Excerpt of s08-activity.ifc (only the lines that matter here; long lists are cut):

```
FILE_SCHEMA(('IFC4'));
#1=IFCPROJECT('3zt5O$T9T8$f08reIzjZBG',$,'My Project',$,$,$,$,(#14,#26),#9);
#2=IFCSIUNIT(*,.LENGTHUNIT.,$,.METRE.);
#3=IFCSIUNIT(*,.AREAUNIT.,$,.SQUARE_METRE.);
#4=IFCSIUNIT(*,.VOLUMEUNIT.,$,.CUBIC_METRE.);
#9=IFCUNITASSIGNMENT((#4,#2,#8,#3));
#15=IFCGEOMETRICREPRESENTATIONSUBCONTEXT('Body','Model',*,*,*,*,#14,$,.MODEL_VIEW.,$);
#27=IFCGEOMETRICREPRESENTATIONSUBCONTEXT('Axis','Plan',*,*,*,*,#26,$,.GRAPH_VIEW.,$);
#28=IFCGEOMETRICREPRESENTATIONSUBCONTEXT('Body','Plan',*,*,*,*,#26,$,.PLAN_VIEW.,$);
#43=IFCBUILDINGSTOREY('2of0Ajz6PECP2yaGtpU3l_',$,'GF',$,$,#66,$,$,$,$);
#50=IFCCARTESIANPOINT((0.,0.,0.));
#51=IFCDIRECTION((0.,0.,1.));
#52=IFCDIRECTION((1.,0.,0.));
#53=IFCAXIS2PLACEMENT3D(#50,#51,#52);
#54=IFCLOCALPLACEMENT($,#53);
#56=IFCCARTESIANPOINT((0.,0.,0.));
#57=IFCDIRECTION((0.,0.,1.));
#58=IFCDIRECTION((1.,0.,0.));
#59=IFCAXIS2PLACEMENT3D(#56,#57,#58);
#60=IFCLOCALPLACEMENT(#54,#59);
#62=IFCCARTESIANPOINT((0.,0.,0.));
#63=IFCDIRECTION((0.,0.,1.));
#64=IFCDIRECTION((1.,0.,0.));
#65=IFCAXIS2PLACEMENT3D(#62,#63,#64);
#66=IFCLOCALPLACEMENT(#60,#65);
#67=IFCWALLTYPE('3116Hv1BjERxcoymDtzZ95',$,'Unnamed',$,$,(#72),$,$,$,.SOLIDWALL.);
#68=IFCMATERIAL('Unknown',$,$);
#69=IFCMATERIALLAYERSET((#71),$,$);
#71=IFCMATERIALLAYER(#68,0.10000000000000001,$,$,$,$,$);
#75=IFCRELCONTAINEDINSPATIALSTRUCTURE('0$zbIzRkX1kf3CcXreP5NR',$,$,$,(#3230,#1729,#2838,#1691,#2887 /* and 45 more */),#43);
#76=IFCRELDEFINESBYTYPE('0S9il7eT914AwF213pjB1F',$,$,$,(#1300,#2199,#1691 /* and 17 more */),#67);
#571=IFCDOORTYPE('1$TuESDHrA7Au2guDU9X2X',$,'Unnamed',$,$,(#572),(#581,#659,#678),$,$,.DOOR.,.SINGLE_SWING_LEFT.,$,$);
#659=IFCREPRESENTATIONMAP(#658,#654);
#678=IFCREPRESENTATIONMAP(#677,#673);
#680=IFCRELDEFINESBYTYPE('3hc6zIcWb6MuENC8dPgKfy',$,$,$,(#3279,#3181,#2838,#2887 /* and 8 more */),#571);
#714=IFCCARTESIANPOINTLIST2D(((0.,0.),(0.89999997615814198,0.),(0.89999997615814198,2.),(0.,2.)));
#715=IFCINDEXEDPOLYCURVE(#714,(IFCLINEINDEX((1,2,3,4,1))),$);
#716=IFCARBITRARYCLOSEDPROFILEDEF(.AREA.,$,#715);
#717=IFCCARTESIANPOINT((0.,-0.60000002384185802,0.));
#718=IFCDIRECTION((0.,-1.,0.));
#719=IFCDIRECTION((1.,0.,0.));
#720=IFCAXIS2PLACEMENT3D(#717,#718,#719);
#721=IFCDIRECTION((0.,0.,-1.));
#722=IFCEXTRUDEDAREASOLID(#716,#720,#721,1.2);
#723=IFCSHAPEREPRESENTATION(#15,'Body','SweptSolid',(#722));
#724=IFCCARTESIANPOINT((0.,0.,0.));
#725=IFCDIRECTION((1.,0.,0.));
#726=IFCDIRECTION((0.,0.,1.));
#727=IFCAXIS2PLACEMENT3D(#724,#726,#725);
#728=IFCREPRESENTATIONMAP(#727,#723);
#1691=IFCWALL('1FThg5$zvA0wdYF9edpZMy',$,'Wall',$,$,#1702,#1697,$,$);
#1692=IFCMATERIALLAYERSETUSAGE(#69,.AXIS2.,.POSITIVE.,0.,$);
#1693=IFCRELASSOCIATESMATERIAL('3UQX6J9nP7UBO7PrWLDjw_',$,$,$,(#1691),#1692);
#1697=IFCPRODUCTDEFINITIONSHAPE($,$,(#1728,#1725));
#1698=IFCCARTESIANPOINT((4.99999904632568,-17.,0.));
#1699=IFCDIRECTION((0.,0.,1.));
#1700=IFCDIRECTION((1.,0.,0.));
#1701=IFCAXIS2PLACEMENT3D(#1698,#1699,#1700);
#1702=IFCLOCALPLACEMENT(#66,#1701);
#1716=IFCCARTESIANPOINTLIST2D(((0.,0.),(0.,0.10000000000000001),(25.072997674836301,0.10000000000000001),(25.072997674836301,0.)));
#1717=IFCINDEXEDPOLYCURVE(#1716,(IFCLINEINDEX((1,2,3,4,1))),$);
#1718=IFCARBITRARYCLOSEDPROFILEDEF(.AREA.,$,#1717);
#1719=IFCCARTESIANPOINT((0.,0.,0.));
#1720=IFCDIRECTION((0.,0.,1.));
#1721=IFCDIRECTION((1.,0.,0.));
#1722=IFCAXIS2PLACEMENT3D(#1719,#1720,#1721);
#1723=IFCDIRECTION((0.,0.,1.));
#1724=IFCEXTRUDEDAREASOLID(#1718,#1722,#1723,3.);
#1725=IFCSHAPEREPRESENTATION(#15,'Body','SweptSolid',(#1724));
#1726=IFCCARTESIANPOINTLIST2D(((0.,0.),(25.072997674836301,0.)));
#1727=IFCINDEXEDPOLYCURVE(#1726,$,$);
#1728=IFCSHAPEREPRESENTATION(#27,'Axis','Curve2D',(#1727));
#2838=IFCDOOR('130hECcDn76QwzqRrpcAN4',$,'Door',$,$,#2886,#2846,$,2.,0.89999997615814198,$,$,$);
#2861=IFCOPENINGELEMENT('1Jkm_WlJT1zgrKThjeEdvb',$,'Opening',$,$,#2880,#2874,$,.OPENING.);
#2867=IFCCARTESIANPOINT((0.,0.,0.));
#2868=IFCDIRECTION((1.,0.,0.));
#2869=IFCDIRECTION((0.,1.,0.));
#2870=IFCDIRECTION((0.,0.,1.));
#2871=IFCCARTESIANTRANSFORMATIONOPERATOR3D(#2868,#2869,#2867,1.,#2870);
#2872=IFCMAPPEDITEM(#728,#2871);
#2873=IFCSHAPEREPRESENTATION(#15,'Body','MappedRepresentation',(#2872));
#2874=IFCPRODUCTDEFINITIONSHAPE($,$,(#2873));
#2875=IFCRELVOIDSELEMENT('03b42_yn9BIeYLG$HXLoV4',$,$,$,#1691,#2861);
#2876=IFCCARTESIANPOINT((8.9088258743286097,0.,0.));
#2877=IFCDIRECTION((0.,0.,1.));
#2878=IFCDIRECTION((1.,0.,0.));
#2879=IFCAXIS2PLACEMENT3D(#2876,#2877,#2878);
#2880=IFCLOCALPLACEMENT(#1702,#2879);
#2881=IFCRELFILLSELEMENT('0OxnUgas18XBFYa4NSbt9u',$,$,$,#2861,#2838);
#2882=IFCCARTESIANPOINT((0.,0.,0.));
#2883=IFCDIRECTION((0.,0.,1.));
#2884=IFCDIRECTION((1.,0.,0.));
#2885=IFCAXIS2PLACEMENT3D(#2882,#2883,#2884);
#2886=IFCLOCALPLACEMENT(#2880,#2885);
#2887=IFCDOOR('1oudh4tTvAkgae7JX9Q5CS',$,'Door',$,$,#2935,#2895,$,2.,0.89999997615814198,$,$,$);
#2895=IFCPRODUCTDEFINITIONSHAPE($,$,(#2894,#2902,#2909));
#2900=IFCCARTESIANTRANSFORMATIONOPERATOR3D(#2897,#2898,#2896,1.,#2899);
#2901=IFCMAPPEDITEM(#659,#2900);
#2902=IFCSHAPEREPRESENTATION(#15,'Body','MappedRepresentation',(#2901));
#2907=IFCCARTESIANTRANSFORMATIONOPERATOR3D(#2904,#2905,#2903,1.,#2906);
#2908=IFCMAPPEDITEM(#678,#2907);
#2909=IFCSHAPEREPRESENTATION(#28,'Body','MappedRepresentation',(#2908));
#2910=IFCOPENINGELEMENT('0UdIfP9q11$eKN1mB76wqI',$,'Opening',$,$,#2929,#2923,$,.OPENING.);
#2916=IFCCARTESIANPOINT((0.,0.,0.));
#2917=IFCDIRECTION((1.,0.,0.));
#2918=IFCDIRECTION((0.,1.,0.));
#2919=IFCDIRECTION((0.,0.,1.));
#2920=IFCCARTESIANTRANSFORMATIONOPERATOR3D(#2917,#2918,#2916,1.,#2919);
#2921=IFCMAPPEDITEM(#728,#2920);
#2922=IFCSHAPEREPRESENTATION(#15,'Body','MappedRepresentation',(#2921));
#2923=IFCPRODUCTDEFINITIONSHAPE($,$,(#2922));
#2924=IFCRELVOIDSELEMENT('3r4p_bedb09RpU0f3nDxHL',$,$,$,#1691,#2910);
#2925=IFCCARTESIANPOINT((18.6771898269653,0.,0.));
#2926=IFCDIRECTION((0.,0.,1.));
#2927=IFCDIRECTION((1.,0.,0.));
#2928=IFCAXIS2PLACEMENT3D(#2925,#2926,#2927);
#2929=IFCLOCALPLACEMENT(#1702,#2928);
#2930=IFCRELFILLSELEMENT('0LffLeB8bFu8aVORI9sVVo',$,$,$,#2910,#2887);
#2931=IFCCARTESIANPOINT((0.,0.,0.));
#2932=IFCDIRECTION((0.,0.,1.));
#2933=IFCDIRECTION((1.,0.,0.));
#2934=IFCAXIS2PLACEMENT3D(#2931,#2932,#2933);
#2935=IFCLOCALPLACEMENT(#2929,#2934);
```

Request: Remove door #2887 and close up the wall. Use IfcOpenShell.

```python
import ifcopenshell
import ifcopenshell.api.feature
import ifcopenshell.api.root
import ifcopenshell.geom
import ifcopenshell.util.shape

model = ifcopenshell.open("s08-activity.ifc")
settings = ifcopenshell.geom.settings()


def volume(element):
    """Net volume in cubic metres, openings subtracted."""
    shape = ifcopenshell.geom.create_shape(settings, element)
    return ifcopenshell.util.shape.get_volume(shape.geometry)


door = model.by_guid("1oudh4tTvAkgae7JX9Q5CS")
opening = door.FillsVoids[0].RelatingOpeningElement
wall = opening.VoidsElements[0].RelatingBuildingElement
before = volume(wall)

ifcopenshell.api.root.remove_product(model, product=door)
ifcopenshell.api.feature.remove_feature(model, feature=opening)

after = volume(wall)

print(f"wall volume {before:.3f} -> {after:.3f} m3")

model.write("s08-activity-out.ifc")
```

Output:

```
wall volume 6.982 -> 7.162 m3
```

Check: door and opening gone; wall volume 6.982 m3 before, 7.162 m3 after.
